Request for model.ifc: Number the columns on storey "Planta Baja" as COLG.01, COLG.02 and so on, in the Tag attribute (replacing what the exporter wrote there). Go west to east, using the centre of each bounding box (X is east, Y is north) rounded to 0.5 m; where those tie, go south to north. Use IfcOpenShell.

First a look at what the model holds.

```python
import ifcopenshell
import ifcopenshell.util.element
import ifcopenshell.util.placement

model = ifcopenshell.open("model.ifc")
print(model.schema)
storey = next(s for s in model.by_type("IfcBuildingStorey") if s.Name == "Planta Baja")
columns = [e for e in ifcopenshell.util.element.get_decomposition(storey) if e.is_a("IfcColumn")]
for e in sorted(columns, key=lambda e: e.id()):
    origin = ifcopenshell.util.placement.get_local_placement(e.ObjectPlacement)[:3, 3]
    print(e.id(), e.Tag, e.Name, origin.round(2) + 0.0, sep=" | ")
```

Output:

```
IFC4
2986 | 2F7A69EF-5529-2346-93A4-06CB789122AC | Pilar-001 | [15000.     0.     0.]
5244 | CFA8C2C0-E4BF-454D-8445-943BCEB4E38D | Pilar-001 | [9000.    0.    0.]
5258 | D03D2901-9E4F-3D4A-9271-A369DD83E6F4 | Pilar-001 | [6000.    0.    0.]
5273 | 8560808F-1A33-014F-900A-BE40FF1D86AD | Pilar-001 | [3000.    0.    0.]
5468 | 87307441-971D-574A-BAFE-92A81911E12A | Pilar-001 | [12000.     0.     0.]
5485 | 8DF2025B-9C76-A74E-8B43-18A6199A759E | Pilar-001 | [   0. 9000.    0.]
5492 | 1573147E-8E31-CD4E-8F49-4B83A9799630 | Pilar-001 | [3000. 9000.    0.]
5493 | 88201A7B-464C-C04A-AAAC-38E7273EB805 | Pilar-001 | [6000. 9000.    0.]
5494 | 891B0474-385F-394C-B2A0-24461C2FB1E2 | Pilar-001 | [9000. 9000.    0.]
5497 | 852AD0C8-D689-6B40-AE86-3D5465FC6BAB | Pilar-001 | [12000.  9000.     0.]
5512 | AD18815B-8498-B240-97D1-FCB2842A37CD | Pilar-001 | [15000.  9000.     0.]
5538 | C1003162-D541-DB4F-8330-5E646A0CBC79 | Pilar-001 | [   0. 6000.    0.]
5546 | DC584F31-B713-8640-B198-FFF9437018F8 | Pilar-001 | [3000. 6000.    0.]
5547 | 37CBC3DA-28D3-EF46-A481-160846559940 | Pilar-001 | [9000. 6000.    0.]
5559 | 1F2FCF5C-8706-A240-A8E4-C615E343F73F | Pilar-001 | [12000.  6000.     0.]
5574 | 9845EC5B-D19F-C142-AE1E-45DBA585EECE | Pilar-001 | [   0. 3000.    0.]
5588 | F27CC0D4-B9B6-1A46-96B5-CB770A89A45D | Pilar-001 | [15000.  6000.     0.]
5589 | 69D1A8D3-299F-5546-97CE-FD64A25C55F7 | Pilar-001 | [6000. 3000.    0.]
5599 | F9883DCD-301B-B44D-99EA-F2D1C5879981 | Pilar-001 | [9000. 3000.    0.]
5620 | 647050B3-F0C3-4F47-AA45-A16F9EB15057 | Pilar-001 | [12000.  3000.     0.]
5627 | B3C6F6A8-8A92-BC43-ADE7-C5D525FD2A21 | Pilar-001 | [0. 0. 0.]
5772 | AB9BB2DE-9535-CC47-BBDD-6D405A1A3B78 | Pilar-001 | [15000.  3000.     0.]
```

```python
import ifcopenshell
import ifcopenshell.geom
import ifcopenshell.util.element
import ifcopenshell.util.shape

model = ifcopenshell.open("model.ifc")
settings = ifcopenshell.geom.settings()
settings.set("use-world-coords", True)


def centre(element):
    shape = ifcopenshell.geom.create_shape(settings, element)
    return ifcopenshell.util.shape.get_bbox_centroid(shape.geometry)


storey = next(s for s in model.by_type("IfcBuildingStorey") if s.Name == "Planta Baja")
columns = [e for e in ifcopenshell.util.element.get_decomposition(storey) if e.is_a("IfcColumn")]

# Insertion points can sit at a corner or the storey origin, so sort by the geometry (in metres).
centres = {e: centre(e) for e in columns}
columns.sort(key=lambda e: (round(centres[e][0] / 0.5), centres[e][1]))

for i, e in enumerate(columns, start=1):
    number = f"COLG.{i:02d}"
    e.Tag = number
    print(e.id(), number)

model.write("model_updated.ifc")
```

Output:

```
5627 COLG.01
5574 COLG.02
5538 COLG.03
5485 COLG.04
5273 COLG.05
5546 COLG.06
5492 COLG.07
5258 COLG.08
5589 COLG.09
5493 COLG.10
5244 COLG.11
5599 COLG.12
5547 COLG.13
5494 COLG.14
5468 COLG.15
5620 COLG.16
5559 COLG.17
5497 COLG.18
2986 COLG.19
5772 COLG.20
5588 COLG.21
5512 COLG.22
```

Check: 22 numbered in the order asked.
